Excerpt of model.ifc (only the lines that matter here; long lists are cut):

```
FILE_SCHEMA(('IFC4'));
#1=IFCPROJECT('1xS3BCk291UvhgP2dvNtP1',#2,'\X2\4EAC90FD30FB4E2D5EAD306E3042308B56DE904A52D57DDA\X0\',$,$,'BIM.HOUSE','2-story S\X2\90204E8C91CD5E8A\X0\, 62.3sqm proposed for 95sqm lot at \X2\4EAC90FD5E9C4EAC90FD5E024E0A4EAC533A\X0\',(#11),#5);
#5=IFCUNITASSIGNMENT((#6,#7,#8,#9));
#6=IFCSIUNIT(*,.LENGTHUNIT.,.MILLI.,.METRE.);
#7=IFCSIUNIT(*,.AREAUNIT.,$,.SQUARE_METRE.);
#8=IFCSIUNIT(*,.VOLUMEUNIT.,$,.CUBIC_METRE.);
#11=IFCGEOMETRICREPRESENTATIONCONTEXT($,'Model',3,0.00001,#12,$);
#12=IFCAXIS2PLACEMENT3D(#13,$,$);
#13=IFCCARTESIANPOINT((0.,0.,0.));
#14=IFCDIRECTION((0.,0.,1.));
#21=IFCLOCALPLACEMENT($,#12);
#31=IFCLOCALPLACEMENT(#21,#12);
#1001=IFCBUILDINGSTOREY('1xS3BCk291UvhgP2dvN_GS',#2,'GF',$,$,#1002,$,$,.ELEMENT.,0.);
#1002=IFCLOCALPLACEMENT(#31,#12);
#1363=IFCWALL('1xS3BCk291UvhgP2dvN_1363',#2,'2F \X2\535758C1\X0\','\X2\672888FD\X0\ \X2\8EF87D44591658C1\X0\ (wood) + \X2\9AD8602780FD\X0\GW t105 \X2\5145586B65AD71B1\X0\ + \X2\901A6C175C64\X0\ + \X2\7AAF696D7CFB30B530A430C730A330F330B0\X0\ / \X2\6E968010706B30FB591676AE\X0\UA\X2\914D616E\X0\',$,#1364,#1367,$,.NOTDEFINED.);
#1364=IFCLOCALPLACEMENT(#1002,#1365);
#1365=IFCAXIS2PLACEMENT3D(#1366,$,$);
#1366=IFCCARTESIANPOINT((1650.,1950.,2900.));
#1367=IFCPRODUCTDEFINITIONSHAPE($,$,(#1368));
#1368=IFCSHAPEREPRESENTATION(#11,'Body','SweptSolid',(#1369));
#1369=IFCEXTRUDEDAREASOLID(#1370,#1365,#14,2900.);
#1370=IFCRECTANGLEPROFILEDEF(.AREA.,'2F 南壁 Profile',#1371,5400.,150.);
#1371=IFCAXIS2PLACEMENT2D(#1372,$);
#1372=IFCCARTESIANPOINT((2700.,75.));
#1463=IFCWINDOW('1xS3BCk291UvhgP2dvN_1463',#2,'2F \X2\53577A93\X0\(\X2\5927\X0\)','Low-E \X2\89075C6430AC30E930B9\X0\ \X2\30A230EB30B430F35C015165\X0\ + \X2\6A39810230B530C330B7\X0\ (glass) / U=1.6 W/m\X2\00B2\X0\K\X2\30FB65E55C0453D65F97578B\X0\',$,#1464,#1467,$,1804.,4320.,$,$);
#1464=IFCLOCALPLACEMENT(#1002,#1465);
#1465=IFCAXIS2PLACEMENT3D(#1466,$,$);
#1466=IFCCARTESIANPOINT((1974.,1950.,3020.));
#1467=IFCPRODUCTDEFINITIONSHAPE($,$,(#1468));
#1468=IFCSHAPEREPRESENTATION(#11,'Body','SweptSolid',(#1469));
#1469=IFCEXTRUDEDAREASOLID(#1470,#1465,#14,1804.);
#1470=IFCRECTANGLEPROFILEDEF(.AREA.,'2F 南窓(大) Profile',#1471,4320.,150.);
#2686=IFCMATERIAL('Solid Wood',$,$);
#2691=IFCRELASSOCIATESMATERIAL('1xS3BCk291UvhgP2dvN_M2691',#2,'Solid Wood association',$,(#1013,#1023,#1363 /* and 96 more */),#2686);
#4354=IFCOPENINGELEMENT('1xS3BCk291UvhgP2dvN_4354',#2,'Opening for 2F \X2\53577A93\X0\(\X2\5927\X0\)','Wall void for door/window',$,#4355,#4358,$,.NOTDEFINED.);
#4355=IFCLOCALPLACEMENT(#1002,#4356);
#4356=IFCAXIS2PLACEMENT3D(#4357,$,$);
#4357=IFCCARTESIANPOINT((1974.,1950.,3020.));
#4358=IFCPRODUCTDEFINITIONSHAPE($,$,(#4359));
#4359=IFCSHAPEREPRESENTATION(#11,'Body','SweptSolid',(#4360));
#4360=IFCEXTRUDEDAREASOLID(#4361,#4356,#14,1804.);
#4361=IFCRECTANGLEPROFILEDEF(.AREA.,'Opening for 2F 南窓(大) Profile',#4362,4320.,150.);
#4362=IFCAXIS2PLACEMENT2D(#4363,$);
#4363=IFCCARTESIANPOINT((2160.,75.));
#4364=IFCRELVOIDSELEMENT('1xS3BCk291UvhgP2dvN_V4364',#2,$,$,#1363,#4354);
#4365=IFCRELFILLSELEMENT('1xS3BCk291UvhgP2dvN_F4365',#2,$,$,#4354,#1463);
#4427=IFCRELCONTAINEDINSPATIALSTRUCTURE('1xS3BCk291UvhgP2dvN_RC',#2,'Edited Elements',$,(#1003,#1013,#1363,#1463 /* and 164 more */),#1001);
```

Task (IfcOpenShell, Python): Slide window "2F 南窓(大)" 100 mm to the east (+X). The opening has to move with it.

```python
import ifcopenshell
import ifcopenshell.api.geometry
import ifcopenshell.util.placement

model = ifcopenshell.open("model.ifc")

window = model.by_guid("1xS3BCk291UvhgP2dvN_1463")
opening = window.FillsVoids[0].RelatingOpeningElement
wall = opening.VoidsElements[0].RelatingBuildingElement

wall_matrix = ifcopenshell.util.placement.get_local_placement(wall.ObjectPlacement)
shift = wall_matrix[:3, 0] * 100.0
before = ifcopenshell.util.placement.get_local_placement(window.ObjectPlacement)[:3, 3].copy()

# The window is not placed relative to its opening, so move both.
for product in (opening, window):
    matrix = ifcopenshell.util.placement.get_local_placement(product.ObjectPlacement)
    matrix[:3, 3] += shift
    ifcopenshell.api.geometry.edit_object_placement(model, product=product, matrix=matrix, is_si=False)

after = ifcopenshell.util.placement.get_local_placement(window.ObjectPlacement)[:3, 3]
print("window moved by", (after - before).round(3) + 0.0)

model.write("model-out.ifc")
```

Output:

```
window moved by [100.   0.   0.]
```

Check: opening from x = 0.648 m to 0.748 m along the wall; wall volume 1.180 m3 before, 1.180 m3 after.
